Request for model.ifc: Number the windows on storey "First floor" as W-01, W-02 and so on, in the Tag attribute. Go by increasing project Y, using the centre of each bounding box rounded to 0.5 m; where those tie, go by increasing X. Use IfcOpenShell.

First a look at what the model holds.

```python
import ifcopenshell
import ifcopenshell.util.element
import ifcopenshell.util.placement

model = ifcopenshell.open("model.ifc")
print(model.schema)
storey = next(s for s in model.by_type("IfcBuildingStorey") if s.Name == "First floor")
windows = [e for e in ifcopenshell.util.element.get_decomposition(storey) if e.is_a("IfcWindow")]
for e in sorted(windows, key=lambda e: e.id()):
    origin = ifcopenshell.util.placement.get_local_placement(e.ObjectPlacement)[:3, 3]
    print(e.id(), e.Tag, e.Name, origin.round(2) + 0.0, sep=" | ")
```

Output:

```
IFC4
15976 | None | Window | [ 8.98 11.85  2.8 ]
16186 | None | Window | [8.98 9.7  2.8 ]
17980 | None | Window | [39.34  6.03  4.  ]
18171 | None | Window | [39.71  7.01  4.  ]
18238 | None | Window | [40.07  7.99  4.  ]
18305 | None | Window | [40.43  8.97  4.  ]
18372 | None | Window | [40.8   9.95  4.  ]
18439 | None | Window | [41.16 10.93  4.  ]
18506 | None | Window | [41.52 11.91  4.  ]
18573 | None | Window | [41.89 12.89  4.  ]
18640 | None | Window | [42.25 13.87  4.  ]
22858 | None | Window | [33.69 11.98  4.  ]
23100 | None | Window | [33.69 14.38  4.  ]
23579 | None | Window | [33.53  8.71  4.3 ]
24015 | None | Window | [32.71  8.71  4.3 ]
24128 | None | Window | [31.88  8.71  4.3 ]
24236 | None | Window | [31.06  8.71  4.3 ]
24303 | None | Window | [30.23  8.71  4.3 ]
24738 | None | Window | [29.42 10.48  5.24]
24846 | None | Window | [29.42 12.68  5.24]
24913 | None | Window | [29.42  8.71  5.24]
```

```python
import ifcopenshell
import ifcopenshell.geom
import ifcopenshell.util.element
import ifcopenshell.util.shape

model = ifcopenshell.open("model.ifc")
settings = ifcopenshell.geom.settings()
settings.set("use-world-coords", True)


def centre(element):
    shape = ifcopenshell.geom.create_shape(settings, element)
    return ifcopenshell.util.shape.get_bbox_centroid(shape.geometry)


storey = next(s for s in model.by_type("IfcBuildingStorey") if s.Name == "First floor")
windows = [e for e in ifcopenshell.util.element.get_decomposition(storey) if e.is_a("IfcWindow")]

# Insertion points can sit at a corner or the storey origin, so sort by the geometry (in metres).
centres = {e: centre(e) for e in windows}
windows.sort(key=lambda e: (round(centres[e][1] / 0.5), centres[e][0]))

for i, e in enumerate(windows, start=1):
    number = f"W-{i:02d}"
    e.Tag = number
    print(e.id(), number)

model.write("model_edited.ifc")
```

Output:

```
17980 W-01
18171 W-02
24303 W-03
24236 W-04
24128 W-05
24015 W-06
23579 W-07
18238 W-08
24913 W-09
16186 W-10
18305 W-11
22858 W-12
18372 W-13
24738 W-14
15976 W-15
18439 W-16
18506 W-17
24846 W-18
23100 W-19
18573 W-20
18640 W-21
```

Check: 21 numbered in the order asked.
